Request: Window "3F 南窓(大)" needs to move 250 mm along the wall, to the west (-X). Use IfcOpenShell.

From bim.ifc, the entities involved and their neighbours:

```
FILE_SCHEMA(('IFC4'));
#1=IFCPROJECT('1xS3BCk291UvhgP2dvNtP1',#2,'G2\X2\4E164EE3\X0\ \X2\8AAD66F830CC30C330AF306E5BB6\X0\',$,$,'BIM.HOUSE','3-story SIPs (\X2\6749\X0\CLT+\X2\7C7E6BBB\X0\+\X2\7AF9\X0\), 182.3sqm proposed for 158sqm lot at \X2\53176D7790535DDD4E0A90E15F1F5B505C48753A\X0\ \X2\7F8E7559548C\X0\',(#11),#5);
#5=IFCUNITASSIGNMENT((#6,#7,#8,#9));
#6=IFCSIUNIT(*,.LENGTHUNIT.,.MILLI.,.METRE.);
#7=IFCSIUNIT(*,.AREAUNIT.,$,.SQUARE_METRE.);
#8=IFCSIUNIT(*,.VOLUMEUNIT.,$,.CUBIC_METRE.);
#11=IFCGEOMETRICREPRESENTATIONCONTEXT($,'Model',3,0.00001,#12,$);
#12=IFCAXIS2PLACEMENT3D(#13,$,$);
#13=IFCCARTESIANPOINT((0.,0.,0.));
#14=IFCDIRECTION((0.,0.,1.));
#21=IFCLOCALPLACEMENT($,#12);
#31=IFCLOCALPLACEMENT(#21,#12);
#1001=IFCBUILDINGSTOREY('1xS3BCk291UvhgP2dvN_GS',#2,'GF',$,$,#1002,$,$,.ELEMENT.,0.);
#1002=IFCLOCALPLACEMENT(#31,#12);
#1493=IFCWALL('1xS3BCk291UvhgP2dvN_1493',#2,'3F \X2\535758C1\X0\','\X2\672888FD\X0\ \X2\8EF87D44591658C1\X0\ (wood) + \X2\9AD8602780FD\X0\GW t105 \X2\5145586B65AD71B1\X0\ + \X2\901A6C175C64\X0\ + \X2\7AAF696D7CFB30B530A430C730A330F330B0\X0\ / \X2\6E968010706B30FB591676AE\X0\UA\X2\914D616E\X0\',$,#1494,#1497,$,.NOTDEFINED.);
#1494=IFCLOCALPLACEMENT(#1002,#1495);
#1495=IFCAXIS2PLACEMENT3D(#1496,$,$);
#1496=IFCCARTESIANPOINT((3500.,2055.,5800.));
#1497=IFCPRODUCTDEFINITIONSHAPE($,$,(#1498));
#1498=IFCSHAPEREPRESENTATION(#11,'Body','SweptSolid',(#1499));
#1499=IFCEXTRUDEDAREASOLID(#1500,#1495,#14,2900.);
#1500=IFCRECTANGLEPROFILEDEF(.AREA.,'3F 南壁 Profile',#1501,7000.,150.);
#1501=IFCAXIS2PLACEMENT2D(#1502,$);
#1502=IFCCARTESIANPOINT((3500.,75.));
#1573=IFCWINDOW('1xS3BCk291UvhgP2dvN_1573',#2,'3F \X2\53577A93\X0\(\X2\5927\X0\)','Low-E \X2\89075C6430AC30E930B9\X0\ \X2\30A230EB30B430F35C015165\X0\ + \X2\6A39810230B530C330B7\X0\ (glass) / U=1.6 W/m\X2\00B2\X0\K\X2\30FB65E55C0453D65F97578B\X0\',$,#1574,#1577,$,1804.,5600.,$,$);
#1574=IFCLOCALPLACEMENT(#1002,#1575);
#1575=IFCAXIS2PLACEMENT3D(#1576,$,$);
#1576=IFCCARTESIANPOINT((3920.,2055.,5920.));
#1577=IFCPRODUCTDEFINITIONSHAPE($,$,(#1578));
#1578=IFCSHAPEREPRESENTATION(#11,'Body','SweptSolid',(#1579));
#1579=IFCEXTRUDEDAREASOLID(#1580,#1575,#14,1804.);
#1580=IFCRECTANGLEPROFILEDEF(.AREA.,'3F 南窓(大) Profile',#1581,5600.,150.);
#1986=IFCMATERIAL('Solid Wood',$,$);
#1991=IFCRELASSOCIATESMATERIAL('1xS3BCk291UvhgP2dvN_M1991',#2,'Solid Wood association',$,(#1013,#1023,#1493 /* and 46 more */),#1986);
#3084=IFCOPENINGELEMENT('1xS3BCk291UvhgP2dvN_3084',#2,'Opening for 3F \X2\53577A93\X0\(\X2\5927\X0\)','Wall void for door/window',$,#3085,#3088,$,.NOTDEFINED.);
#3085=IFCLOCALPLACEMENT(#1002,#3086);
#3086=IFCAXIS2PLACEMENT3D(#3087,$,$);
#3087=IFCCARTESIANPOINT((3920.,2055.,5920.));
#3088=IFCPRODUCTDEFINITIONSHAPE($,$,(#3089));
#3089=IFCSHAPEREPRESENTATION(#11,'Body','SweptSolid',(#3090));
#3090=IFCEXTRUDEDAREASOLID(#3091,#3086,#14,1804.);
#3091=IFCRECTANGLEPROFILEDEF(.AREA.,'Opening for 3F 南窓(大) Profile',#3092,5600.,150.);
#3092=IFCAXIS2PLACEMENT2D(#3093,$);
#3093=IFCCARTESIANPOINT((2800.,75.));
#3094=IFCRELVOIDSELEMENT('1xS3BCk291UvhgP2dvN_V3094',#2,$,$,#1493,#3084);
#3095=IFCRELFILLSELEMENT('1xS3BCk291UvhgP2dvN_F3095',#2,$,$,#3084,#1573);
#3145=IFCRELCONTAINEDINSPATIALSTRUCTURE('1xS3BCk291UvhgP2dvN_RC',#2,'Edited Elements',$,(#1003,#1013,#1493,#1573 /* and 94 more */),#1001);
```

```python
import ifcopenshell
import ifcopenshell.api.geometry
import ifcopenshell.util.placement
import ifcopenshell.util.unit

model = ifcopenshell.open("bim.ifc")
unit_scale = ifcopenshell.util.unit.calculate_unit_scale(model)

window = model.by_id(1573)
opening = window.FillsVoids[0].RelatingOpeningElement
wall = opening.VoidsElements[0].RelatingBuildingElement

wall_matrix = ifcopenshell.util.placement.get_local_placement(wall.ObjectPlacement)
shift = wall_matrix[:3, 0] * -0.25 / unit_scale
before = ifcopenshell.util.placement.get_local_placement(window.ObjectPlacement)[:3, 3].copy()

# The window is not placed relative to its opening, so move both.
for product in (opening, window):
    matrix = ifcopenshell.util.placement.get_local_placement(product.ObjectPlacement)
    matrix[:3, 3] += shift
    ifcopenshell.api.geometry.edit_object_placement(model, product=product, matrix=matrix, is_si=False)

after = ifcopenshell.util.placement.get_local_placement(window.ObjectPlacement)[:3, 3]
print("window moved by", (after - before).round(3) + 0.0)

model.write("bim_v2.ifc")
```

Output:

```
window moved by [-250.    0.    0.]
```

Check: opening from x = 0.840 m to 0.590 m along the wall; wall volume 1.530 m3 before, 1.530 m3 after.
